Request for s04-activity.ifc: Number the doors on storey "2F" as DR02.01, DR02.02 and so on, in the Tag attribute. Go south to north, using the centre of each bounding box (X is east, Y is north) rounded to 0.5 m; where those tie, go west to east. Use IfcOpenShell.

First a look at what the model holds.

```python
import ifcopenshell
import ifcopenshell.util.element
import ifcopenshell.util.placement

model = ifcopenshell.open("s04-activity.ifc")
print(model.schema)
storey = next(s for s in model.by_type("IfcBuildingStorey") if s.Name == "2F")
doors = [e for e in ifcopenshell.util.element.get_decomposition(storey) if e.is_a("IfcDoor")]
for e in sorted(doors, key=lambda e: e.id()):
    origin = ifcopenshell.util.placement.get_local_placement(e.ObjectPlacement)[:3, 3]
    print(e.id(), e.Tag, e.Name, origin.round(2) + 0.0, sep=" | ")
```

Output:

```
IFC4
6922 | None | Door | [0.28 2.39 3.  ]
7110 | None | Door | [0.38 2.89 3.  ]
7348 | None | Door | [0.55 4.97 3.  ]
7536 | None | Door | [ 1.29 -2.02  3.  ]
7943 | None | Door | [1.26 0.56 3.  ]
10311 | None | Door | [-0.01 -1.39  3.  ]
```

```python
import ifcopenshell
import ifcopenshell.geom
import ifcopenshell.util.element
import ifcopenshell.util.shape

model = ifcopenshell.open("s04-activity.ifc")
settings = ifcopenshell.geom.settings()
settings.set("use-world-coords", True)


def centre(element):
    shape = ifcopenshell.geom.create_shape(settings, element)
    return ifcopenshell.util.shape.get_bbox_centroid(shape.geometry)


storey = next(s for s in model.by_type("IfcBuildingStorey") if s.Name == "2F")
doors = [e for e in ifcopenshell.util.element.get_decomposition(storey) if e.is_a("IfcDoor")]

# Insertion points can sit at a corner or the storey origin, so sort by the geometry (in metres).
centres = {e: centre(e) for e in doors}
doors.sort(key=lambda e: (round(centres[e][1] / 0.5), centres[e][0]))

for i, e in enumerate(doors, start=1):
    number = f"DR02.{i:02d}"
    e.Tag = number
    print(e.id(), number)

model.write("s04-activity_rev.ifc")
```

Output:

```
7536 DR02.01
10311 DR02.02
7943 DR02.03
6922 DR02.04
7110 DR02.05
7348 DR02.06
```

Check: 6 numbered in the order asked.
